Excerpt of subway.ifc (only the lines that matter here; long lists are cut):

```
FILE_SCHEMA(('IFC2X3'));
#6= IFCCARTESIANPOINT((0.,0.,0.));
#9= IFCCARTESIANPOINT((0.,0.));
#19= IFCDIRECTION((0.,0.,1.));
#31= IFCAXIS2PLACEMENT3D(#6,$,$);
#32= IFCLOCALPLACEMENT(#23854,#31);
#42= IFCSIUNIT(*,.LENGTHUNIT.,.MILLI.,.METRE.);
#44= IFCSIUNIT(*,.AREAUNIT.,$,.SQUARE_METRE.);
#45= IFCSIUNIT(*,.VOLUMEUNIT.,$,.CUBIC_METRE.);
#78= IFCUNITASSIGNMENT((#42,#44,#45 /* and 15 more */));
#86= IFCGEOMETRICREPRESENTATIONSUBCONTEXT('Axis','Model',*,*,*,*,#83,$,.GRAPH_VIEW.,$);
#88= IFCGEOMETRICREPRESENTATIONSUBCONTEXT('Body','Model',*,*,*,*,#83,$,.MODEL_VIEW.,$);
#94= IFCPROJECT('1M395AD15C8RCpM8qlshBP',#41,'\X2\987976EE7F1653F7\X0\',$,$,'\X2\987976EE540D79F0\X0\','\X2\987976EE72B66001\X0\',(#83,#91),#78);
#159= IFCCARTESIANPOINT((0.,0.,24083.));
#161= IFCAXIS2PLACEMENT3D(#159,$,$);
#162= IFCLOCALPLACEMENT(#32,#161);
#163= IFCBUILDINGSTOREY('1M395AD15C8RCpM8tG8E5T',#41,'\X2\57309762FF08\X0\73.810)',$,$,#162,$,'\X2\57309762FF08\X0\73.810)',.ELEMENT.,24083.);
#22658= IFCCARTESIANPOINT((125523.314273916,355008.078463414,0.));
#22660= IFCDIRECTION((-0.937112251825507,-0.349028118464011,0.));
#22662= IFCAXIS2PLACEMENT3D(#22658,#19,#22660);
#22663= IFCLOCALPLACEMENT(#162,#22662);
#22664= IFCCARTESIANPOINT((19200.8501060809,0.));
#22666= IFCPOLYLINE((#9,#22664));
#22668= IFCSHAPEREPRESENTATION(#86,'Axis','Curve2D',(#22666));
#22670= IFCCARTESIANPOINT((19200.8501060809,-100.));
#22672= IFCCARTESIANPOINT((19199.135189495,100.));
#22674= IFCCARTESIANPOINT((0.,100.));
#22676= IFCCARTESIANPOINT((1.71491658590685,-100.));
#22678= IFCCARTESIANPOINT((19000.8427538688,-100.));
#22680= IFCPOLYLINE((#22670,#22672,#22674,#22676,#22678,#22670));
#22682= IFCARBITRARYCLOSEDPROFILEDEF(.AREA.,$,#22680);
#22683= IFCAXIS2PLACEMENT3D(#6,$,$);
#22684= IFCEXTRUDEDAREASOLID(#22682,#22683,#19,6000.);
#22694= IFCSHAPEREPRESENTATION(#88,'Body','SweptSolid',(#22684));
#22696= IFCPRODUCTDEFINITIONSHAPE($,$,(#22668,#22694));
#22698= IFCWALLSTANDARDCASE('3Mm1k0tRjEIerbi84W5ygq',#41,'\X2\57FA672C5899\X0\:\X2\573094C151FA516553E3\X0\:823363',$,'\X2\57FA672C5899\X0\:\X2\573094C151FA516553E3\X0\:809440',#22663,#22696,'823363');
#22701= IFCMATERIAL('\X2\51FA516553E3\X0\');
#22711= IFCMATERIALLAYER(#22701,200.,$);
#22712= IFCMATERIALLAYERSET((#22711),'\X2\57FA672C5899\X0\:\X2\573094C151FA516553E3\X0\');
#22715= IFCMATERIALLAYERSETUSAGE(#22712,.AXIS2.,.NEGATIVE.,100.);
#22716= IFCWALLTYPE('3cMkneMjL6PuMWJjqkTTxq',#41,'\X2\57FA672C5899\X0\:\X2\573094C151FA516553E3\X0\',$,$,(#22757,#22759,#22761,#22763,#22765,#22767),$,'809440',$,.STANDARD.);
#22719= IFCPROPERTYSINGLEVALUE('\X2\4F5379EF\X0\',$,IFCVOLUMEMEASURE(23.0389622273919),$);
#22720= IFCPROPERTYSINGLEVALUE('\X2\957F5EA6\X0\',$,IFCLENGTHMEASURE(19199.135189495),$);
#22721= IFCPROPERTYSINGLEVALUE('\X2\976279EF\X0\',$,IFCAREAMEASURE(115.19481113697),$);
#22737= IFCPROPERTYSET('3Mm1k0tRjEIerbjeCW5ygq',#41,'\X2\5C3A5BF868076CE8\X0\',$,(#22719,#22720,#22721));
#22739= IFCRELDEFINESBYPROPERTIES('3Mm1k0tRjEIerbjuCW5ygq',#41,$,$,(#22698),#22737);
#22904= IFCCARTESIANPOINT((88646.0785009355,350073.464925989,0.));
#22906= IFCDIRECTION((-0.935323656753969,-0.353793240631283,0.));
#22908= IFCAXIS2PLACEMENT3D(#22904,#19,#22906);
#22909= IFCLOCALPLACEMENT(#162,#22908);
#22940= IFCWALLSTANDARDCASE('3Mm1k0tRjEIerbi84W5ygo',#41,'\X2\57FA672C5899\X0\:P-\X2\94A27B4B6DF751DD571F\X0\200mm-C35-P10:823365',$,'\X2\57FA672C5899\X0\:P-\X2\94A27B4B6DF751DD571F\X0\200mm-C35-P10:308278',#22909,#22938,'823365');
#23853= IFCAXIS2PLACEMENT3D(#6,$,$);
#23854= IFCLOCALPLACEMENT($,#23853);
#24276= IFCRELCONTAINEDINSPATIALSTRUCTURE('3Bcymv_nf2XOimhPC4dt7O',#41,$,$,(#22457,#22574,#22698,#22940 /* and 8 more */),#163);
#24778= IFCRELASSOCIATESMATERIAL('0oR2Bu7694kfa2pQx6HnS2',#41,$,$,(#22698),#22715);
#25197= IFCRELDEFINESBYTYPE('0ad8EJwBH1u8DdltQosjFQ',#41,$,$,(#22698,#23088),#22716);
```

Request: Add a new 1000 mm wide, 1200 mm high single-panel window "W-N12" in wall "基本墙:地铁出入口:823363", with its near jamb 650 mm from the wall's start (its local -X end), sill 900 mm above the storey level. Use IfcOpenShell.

```python
import numpy as np
import ifcopenshell
import ifcopenshell.api.feature
import ifcopenshell.api.geometry
import ifcopenshell.api.pset
import ifcopenshell.api.root
import ifcopenshell.api.spatial
import ifcopenshell.api.type
import ifcopenshell.geom
import ifcopenshell.util.element
import ifcopenshell.util.placement
import ifcopenshell.util.representation
import ifcopenshell.util.shape
import ifcopenshell.util.unit

model = ifcopenshell.open("subway.ifc")
unit_scale = ifcopenshell.util.unit.calculate_unit_scale(model)
area_scale = ifcopenshell.util.unit.calculate_unit_scale(model, "AREAUNIT")
volume_scale = ifcopenshell.util.unit.calculate_unit_scale(model, "VOLUMEUNIT")
settings = ifcopenshell.geom.settings()


def volume(element):
    """Net volume in cubic metres, openings subtracted."""
    shape = ifcopenshell.geom.create_shape(settings, element)
    return ifcopenshell.util.shape.get_volume(shape.geometry)


wall = model.by_guid("3Mm1k0tRjEIerbi84W5ygq")
storey = ifcopenshell.util.element.get_container(wall, ifc_class="IfcBuildingStorey")
context = ifcopenshell.util.representation.get_context(model, "Model", "Body", "MODEL_VIEW")
before = volume(wall)

width, height, from_end, sill = 1, 1.2, 0.65, 0.9  # metres

# The wall runs along its own X axis, and the end named is its -X end.
wall_shape = ifcopenshell.geom.create_shape(settings, wall)
x, y, z = ifcopenshell.util.shape.get_vertices(wall_shape.geometry).T
start = x.min() + from_end
face, thickness = float(y.min()), float(y.max() - y.min())
wall_matrix = ifcopenshell.util.placement.get_local_placement(wall.ObjectPlacement)
level = ifcopenshell.util.placement.get_local_placement(storey.ObjectPlacement)[2, 3]


def in_wall(x, y):
    """Placement at x, y metres in the wall's axes, at sill height."""
    matrix = wall_matrix.copy()
    matrix[:, 3] = wall_matrix @ np.array([x / unit_scale, y / unit_scale, 0.0, 1.0])
    matrix[2, 3] = level + sill / unit_scale
    return matrix


# Opening: a box that overshoots both wall faces by 50 mm.
opening = ifcopenshell.api.root.create_entity(model, ifc_class="IfcOpeningElement")
box = ifcopenshell.api.geometry.add_wall_representation(
    model, context=context, length=width, height=height, thickness=thickness + 0.1
)
ifcopenshell.api.geometry.assign_representation(model, product=opening, representation=box)
ifcopenshell.api.geometry.edit_object_placement(model, product=opening, matrix=in_wall(start, face - 0.05), is_si=False)
ifcopenshell.api.feature.add_feature(model, feature=opening, element=wall)

window = ifcopenshell.api.root.create_entity(model, ifc_class="IfcWindow", name="W-N12")
window.OverallWidth, window.OverallHeight = width / unit_scale, height / unit_scale
body = ifcopenshell.api.geometry.add_window_representation(
    model,
    context=context,
    overall_width=window.OverallWidth,
    overall_height=window.OverallHeight,
    partition_type="SINGLE_PANEL",
)
ifcopenshell.api.geometry.assign_representation(model, product=window, representation=body)
ifcopenshell.api.spatial.assign_container(model, products=[window], relating_structure=storey)
fills = ifcopenshell.api.feature.add_filling(model, opening=opening, element=window)
fills.OwnerHistory = window.OwnerHistory  # required in IFC2X3

# IFC2X3 keeps the operation on the window style.
style = ifcopenshell.api.root.create_entity(model, ifc_class="IfcWindowStyle", name="W-N12")
style.OperationType, style.ConstructionType = "SINGLE_PANEL", "NOTDEFINED"
style.ParameterTakesPrecedence = style.Sizeable = False
ifcopenshell.api.type.assign_type(model, related_objects=[window], relating_type=style)

# Centre the window in the wall's thickness.
ifcopenshell.api.geometry.edit_object_placement(model, product=window, matrix=in_wall(start, face), is_si=False)
window_shape = ifcopenshell.geom.create_shape(settings, window)
depth = ifcopenshell.util.shape.get_vertices(window_shape.geometry)[:, 1]
offset = face + thickness / 2 - (depth.min() + depth.max()) / 2
ifcopenshell.api.geometry.edit_object_placement(model, product=window, matrix=in_wall(start, offset), is_si=False)

after = volume(wall)

# Update the wall's stored quantities.
pset = model.by_id(ifcopenshell.util.element.get_pset(wall, "尺寸标注", should_inherit=False)["id"])
ifcopenshell.api.pset.edit_pset(model, pset=pset, properties={
    "体积": model.create_entity("IfcVolumeMeasure", after / volume_scale),
    "面积": model.create_entity("IfcAreaMeasure", after / thickness / area_scale),
})

print(f"wall volume {before:.3f} -> {after:.3f} m3")

model.write("subway_rev.ifc")
```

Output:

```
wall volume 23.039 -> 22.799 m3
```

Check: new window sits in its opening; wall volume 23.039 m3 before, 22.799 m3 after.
